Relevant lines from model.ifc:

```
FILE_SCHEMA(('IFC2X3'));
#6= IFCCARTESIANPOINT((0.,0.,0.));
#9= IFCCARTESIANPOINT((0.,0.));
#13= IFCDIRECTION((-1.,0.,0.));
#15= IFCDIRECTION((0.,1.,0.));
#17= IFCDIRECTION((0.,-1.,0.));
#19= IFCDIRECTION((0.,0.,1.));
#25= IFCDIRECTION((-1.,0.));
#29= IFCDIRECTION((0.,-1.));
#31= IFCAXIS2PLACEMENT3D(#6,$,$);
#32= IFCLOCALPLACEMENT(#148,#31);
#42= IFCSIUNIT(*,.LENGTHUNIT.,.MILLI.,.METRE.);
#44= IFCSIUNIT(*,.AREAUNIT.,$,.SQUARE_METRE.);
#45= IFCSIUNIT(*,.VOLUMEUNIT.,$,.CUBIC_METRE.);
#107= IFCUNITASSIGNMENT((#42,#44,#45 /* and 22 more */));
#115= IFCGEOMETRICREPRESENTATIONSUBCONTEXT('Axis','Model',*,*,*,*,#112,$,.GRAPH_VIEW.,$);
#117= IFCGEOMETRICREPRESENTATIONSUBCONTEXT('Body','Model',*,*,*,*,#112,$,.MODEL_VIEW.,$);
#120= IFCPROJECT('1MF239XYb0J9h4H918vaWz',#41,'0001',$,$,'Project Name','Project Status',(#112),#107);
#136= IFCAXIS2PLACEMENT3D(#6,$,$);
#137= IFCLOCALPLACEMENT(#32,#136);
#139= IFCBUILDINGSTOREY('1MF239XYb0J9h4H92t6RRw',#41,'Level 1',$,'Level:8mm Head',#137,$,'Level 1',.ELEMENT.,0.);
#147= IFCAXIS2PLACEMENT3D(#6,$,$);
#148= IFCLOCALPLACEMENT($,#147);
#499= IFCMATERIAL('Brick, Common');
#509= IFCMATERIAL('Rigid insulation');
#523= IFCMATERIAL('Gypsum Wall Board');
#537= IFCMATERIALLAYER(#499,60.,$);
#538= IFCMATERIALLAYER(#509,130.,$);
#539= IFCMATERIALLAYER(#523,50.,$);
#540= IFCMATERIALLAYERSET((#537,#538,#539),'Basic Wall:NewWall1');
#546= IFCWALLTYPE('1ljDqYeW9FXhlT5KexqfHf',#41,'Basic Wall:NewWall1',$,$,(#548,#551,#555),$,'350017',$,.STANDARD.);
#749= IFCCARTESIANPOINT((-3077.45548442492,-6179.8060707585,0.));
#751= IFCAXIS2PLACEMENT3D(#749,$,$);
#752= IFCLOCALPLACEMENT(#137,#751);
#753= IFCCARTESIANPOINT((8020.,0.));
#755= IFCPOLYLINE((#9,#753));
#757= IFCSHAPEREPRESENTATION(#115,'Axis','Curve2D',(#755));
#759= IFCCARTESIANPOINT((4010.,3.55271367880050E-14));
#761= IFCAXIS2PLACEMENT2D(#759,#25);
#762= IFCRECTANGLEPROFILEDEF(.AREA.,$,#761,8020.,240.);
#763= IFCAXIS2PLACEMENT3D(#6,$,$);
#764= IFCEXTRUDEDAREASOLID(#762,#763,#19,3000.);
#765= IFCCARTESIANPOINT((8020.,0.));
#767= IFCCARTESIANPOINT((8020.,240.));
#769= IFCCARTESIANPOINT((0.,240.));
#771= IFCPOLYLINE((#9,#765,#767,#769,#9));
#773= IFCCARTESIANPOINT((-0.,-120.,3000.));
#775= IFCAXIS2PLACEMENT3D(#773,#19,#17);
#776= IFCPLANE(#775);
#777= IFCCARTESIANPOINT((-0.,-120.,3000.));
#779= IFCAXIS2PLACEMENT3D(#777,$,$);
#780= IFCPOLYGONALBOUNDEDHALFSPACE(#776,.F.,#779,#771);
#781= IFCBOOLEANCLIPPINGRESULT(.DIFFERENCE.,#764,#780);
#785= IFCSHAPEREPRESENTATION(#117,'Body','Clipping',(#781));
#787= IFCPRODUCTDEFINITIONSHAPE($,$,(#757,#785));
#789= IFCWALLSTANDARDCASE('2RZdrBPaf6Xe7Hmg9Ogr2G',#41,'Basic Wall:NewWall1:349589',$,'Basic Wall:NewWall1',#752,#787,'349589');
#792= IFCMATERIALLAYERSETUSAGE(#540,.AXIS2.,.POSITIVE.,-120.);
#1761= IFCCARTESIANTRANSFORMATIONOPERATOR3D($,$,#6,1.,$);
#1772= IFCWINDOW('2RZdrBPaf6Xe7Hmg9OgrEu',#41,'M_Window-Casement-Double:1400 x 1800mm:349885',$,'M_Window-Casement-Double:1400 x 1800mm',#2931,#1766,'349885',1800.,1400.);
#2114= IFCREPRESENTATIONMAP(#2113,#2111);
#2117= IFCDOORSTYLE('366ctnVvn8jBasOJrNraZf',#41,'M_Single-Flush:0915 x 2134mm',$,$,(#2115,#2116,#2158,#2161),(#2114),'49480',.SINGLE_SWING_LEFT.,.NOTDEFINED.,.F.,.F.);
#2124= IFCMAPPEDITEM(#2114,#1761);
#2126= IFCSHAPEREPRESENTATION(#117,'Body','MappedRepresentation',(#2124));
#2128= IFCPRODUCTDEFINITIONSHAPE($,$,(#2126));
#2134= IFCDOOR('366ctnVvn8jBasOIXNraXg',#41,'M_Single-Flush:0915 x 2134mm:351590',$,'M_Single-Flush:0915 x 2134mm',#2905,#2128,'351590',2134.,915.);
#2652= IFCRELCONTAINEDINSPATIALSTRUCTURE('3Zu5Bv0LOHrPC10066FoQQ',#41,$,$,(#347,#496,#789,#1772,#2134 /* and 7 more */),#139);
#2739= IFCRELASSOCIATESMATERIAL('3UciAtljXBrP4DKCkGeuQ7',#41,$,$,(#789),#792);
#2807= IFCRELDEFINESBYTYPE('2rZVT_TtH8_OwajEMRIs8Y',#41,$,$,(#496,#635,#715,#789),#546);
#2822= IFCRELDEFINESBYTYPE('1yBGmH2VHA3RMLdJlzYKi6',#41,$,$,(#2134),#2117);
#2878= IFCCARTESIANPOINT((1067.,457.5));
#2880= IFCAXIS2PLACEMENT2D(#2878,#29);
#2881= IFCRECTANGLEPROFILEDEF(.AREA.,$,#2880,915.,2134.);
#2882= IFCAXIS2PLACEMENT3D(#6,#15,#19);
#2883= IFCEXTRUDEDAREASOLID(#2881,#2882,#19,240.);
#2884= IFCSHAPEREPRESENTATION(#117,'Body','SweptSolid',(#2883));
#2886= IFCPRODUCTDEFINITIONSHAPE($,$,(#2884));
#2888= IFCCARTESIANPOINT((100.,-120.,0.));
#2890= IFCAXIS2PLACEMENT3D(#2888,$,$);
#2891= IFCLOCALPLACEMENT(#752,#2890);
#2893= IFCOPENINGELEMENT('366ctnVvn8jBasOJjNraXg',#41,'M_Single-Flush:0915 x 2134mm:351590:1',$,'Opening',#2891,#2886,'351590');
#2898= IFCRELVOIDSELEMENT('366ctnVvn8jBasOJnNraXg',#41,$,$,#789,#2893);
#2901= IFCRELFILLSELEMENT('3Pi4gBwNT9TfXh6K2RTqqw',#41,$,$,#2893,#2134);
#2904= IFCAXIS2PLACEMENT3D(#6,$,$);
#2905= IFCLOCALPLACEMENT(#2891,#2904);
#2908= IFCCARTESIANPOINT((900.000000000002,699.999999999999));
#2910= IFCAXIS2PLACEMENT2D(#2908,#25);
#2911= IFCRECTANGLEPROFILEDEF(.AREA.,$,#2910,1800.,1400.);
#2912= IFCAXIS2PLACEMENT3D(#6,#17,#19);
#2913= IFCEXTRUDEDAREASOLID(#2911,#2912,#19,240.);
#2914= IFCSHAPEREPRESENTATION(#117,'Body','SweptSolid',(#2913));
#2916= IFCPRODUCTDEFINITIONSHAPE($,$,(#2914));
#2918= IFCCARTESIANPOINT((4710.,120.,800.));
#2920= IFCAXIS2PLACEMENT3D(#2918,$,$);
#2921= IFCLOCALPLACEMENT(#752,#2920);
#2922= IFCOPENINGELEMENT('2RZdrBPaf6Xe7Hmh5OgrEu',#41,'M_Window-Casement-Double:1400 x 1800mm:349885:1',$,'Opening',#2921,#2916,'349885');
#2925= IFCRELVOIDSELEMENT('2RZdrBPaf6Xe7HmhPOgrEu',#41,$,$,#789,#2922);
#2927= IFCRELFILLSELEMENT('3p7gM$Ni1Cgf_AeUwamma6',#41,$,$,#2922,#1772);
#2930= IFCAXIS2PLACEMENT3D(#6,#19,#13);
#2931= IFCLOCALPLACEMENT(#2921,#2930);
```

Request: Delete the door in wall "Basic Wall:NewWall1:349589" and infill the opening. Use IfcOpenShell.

```python
import ifcopenshell
import ifcopenshell.api.feature
import ifcopenshell.api.root
import ifcopenshell.geom
import ifcopenshell.util.shape

model = ifcopenshell.open("model.ifc")
settings = ifcopenshell.geom.settings()


def volume(element):
    """Net volume in cubic metres, openings subtracted."""
    shape = ifcopenshell.geom.create_shape(settings, element)
    return ifcopenshell.util.shape.get_volume(shape.geometry)


door = model.by_id(2134)
opening = door.FillsVoids[0].RelatingOpeningElement
wall = opening.VoidsElements[0].RelatingBuildingElement
before = volume(wall)

ifcopenshell.api.root.remove_product(model, product=door)
ifcopenshell.api.feature.remove_feature(model, feature=opening)

after = volume(wall)

print(f"wall volume {before:.3f} -> {after:.3f} m3")

model.write("model_edited.ifc")
```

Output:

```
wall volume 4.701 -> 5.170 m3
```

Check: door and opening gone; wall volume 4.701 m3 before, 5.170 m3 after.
